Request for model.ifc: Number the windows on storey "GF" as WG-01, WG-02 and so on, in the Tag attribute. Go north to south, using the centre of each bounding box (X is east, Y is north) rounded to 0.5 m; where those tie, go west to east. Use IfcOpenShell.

First a look at what the model holds.

```python
import ifcopenshell
import ifcopenshell.util.element
import ifcopenshell.util.placement

model = ifcopenshell.open("model.ifc")
print(model.schema)
storey = next(s for s in model.by_type("IfcBuildingStorey") if s.Name == "GF")
windows = [e for e in ifcopenshell.util.element.get_decomposition(storey) if e.is_a("IfcWindow")]
for e in sorted(windows, key=lambda e: e.id()):
    origin = ifcopenshell.util.placement.get_local_placement(e.ObjectPlacement)[:3, 3]
    print(e.id(), e.Tag, e.Name, origin.round(2) + 0.0, sep=" | ")
```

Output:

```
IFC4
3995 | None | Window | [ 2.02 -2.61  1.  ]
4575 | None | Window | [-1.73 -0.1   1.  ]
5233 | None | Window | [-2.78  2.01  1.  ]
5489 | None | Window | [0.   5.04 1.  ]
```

```python
import ifcopenshell
import ifcopenshell.geom
import ifcopenshell.util.element
import ifcopenshell.util.shape

model = ifcopenshell.open("model.ifc")
settings = ifcopenshell.geom.settings()
settings.set("use-world-coords", True)


def centre(element):
    shape = ifcopenshell.geom.create_shape(settings, element)
    return ifcopenshell.util.shape.get_bbox_centroid(shape.geometry)


storey = next(s for s in model.by_type("IfcBuildingStorey") if s.Name == "GF")
windows = [e for e in ifcopenshell.util.element.get_decomposition(storey) if e.is_a("IfcWindow")]

# Insertion points can sit at a corner or the storey origin, so sort by the geometry (in metres).
centres = {e: centre(e) for e in windows}
windows.sort(key=lambda e: (-round(centres[e][1] / 0.5), centres[e][0]))

for i, e in enumerate(windows, start=1):
    number = f"WG-{i:02d}"
    e.Tag = number
    print(e.id(), number)

model.write("model_rev.ifc")
```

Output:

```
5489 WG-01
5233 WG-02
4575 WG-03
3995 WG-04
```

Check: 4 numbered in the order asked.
